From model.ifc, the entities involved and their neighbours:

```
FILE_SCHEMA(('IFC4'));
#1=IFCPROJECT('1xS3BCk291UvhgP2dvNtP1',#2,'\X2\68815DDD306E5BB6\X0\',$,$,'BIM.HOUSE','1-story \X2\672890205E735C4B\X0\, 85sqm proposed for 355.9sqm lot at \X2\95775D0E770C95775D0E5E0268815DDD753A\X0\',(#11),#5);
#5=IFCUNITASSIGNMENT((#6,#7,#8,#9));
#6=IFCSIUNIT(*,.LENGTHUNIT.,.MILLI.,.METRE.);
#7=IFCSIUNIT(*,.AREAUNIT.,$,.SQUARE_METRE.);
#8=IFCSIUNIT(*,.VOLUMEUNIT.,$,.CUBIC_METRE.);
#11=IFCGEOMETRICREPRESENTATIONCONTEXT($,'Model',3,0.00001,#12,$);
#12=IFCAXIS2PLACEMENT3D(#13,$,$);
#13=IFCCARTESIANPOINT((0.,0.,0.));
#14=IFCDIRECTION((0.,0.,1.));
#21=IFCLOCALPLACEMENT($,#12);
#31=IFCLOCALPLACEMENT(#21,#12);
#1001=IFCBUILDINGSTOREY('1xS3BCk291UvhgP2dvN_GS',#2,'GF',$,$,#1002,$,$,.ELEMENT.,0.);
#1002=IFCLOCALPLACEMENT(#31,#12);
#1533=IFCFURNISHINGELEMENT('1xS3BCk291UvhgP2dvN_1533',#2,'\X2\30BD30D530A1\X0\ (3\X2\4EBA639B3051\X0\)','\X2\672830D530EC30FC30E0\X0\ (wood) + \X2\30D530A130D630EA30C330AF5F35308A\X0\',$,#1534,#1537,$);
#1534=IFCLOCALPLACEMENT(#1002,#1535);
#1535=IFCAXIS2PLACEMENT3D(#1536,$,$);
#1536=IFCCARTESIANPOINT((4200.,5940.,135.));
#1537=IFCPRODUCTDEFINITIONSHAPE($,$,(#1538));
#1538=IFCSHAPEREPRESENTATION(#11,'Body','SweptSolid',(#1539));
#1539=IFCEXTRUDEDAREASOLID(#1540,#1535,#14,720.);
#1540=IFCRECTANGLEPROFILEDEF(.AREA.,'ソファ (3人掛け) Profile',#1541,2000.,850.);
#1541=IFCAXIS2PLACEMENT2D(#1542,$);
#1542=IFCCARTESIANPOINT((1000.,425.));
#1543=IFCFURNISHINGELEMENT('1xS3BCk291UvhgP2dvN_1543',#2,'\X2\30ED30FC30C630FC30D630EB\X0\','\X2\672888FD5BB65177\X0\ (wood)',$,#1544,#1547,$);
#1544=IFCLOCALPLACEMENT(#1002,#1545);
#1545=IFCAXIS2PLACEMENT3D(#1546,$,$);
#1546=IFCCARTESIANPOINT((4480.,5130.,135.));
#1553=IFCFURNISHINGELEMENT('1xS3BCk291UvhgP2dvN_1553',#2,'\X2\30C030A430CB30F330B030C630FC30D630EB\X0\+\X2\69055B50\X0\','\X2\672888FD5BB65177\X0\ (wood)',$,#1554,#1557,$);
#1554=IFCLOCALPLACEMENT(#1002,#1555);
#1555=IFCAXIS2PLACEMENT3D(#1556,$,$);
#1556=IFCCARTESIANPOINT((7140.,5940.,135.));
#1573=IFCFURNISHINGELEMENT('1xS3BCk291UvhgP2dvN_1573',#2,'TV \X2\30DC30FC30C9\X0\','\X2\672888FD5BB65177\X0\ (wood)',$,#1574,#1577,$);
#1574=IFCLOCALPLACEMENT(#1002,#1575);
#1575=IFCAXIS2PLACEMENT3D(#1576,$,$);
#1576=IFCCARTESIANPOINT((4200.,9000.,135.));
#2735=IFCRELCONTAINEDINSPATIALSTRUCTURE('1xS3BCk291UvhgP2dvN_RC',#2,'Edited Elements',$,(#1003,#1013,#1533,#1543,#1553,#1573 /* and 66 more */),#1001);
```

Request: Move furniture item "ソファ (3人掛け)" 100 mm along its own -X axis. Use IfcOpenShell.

```python
import ifcopenshell
import ifcopenshell.api.geometry
import ifcopenshell.util.placement
import ifcopenshell.util.unit

model = ifcopenshell.open("model.ifc")
unit_scale = ifcopenshell.util.unit.calculate_unit_scale(model)

item = model.by_guid("1xS3BCk291UvhgP2dvN_1533")
matrix = ifcopenshell.util.placement.get_local_placement(item.ObjectPlacement)
matrix[:3, 3] -= matrix[:3, 0] * 0.1 / unit_scale
ifcopenshell.api.geometry.edit_object_placement(model, product=item, matrix=matrix, is_si=False)

print(ifcopenshell.util.placement.get_local_placement(item.ObjectPlacement).round(3) + 0.0)

model.write("model_v2.ifc")
```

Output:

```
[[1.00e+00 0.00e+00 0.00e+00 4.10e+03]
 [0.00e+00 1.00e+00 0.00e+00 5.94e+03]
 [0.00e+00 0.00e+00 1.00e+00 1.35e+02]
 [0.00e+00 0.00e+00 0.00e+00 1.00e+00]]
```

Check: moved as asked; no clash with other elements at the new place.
